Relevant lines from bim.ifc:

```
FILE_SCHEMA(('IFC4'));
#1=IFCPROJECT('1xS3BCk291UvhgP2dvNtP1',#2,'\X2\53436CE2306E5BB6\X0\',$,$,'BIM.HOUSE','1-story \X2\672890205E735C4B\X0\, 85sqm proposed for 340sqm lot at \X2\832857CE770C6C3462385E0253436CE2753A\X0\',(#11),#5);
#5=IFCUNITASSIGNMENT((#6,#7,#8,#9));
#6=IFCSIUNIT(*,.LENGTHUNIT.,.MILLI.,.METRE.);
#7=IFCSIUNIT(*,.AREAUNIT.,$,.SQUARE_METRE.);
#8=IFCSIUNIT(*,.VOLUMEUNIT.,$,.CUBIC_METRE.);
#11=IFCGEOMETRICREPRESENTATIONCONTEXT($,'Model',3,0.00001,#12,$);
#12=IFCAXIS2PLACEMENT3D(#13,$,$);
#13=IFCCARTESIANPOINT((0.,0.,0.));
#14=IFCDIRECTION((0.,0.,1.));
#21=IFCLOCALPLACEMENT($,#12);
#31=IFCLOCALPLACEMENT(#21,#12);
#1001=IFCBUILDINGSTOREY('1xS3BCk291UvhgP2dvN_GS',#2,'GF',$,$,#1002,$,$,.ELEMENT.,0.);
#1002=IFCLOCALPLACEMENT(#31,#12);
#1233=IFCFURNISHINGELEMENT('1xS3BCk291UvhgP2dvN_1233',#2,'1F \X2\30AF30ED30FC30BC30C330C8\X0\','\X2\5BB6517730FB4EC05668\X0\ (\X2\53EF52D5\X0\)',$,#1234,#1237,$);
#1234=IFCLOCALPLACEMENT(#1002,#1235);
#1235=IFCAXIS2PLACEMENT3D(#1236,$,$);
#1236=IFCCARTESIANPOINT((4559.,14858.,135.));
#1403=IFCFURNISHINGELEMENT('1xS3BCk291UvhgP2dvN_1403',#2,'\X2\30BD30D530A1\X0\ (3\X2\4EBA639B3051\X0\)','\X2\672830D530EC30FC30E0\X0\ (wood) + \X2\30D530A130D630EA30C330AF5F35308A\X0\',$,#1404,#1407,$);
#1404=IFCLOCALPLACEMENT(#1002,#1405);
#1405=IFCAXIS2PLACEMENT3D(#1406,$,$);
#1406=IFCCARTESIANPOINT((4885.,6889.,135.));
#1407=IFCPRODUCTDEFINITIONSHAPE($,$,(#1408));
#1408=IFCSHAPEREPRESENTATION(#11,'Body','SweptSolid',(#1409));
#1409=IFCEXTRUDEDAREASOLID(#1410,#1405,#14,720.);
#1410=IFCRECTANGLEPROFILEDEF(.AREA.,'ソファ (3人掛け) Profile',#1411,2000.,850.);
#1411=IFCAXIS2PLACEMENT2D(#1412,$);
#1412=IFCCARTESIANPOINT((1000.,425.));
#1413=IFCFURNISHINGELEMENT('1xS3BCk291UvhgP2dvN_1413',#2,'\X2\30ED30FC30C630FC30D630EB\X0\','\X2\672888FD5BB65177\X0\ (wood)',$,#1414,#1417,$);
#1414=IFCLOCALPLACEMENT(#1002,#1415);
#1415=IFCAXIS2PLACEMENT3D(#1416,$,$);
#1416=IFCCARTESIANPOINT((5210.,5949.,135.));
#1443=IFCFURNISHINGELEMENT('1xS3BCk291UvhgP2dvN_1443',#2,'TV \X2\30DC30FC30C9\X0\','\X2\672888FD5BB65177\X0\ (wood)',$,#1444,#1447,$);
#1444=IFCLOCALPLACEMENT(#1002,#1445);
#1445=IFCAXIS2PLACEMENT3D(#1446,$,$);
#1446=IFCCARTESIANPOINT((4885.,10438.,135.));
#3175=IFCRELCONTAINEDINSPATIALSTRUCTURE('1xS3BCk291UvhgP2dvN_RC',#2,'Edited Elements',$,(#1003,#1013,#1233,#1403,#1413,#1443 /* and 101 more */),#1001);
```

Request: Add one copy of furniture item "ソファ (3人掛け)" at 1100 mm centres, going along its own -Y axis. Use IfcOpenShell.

```python
import ifcopenshell
import ifcopenshell.api.geometry
import ifcopenshell.api.root
import ifcopenshell.util.element
import ifcopenshell.util.placement
import ifcopenshell.util.unit

model = ifcopenshell.open("bim.ifc")
unit_scale = ifcopenshell.util.unit.calculate_unit_scale(model)


def reuse_history(source, copy):
    """copy_class also copies each property set's owner history, people and application; keep the originals."""
    for rel in copy.IsDefinedBy:
        if rel.is_a("IfcRelDefinesByProperties") and (history := rel.RelatingPropertyDefinition.OwnerHistory):
            rel.RelatingPropertyDefinition.OwnerHistory = source.OwnerHistory
            ifcopenshell.util.element.remove_deep2(model, history)


source = model.by_guid("1xS3BCk291UvhgP2dvN_1403")
base = ifcopenshell.util.placement.get_local_placement(source.ObjectPlacement)
step = -base[:3, 1] * 1.1 / unit_scale

for i in range(1, 2):
    copy = ifcopenshell.api.root.copy_class(model, product=source)
    copy.Representation = ifcopenshell.util.element.copy_deep(
        model, source.Representation, exclude=["IfcGeometricRepresentationContext", "IfcRepresentationMap"]
    )
    reuse_history(source, copy)
    matrix = base.copy()
    matrix[:3, 3] += i * step
    print("added at", matrix[:3, 3].round(3) + 0.0)
    ifcopenshell.api.geometry.edit_object_placement(model, product=copy, matrix=matrix, is_si=False)

model.write("bim_v2.ifc")
```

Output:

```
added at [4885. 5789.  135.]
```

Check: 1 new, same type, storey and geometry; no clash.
